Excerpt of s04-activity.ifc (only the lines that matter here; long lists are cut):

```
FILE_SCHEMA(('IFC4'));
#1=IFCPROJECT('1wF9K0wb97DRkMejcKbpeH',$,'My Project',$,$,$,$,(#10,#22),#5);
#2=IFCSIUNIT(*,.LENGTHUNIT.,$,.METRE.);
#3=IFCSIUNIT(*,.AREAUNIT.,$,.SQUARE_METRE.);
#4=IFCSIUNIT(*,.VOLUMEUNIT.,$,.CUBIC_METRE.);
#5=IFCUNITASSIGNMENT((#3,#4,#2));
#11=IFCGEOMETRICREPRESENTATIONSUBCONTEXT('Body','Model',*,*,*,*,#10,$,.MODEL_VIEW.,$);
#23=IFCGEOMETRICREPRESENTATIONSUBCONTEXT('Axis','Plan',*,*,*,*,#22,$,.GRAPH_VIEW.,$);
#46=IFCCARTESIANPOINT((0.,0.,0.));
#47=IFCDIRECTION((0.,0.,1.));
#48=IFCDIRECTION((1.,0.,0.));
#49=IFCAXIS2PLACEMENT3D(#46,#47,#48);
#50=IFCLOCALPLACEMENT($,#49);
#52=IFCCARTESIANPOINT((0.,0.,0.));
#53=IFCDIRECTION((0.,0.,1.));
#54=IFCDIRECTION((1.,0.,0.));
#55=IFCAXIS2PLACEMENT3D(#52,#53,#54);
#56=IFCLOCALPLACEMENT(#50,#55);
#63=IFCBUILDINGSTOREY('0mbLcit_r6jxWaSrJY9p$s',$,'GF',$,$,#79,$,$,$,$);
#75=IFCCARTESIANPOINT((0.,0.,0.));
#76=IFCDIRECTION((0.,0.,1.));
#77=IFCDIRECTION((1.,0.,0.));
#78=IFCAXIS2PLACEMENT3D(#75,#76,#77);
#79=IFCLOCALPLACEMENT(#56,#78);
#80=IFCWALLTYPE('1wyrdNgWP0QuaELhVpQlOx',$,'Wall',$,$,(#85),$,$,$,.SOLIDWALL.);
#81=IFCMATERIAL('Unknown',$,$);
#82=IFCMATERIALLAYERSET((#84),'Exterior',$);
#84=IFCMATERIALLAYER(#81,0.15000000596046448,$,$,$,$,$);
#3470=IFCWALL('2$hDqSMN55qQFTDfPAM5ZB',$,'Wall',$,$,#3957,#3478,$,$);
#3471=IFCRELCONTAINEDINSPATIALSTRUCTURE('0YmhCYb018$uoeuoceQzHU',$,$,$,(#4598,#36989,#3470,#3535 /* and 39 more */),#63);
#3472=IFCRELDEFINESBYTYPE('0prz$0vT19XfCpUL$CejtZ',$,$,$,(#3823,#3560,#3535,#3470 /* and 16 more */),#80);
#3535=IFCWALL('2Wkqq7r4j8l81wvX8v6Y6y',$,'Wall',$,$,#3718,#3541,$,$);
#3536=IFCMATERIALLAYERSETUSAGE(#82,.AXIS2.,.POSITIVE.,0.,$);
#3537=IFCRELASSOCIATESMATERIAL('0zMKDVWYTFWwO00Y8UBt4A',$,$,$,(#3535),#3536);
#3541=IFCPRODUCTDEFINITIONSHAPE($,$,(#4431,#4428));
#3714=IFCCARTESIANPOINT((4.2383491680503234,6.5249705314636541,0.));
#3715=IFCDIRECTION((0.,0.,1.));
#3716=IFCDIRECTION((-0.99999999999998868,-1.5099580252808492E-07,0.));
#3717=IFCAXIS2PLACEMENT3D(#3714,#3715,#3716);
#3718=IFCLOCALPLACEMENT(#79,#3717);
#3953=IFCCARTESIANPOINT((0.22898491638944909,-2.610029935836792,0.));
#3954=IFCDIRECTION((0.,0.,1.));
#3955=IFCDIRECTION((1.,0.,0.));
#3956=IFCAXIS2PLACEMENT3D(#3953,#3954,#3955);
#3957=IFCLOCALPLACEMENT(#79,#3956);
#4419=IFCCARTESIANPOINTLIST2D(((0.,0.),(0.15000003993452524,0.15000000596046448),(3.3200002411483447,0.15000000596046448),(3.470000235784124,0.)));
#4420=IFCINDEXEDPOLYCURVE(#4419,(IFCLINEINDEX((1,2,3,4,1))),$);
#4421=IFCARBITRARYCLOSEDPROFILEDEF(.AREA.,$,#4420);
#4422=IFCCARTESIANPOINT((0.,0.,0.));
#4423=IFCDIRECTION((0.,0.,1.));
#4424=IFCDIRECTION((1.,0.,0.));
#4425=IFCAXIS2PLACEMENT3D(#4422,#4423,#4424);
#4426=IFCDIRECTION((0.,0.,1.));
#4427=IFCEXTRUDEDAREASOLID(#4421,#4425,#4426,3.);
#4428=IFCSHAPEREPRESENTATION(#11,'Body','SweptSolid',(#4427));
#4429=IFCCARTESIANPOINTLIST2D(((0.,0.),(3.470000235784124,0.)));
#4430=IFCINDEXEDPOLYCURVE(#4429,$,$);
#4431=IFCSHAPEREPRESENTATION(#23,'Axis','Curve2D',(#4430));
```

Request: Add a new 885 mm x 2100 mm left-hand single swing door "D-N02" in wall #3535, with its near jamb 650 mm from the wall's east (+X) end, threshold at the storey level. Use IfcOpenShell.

```python
import numpy as np
import ifcopenshell
import ifcopenshell.api.feature
import ifcopenshell.api.geometry
import ifcopenshell.api.root
import ifcopenshell.api.spatial
import ifcopenshell.geom
import ifcopenshell.util.element
import ifcopenshell.util.placement
import ifcopenshell.util.representation
import ifcopenshell.util.shape
import ifcopenshell.util.unit

model = ifcopenshell.open("s04-activity.ifc")
unit_scale = ifcopenshell.util.unit.calculate_unit_scale(model)
settings = ifcopenshell.geom.settings()


def volume(element):
    """Net volume in cubic metres, openings subtracted."""
    shape = ifcopenshell.geom.create_shape(settings, element)
    return ifcopenshell.util.shape.get_volume(shape.geometry)


wall = model.by_guid("2Wkqq7r4j8l81wvX8v6Y6y")
storey = ifcopenshell.util.element.get_container(wall, ifc_class="IfcBuildingStorey")
context = ifcopenshell.util.representation.get_context(model, "Model", "Body", "MODEL_VIEW")
before = volume(wall)

width, height, from_end, sill = 0.885, 2.1, 0.65, 0.0  # metres

# The wall runs along its own X axis, and the end named is its -X end.
wall_shape = ifcopenshell.geom.create_shape(settings, wall)
x, y, z = ifcopenshell.util.shape.get_vertices(wall_shape.geometry).T
start = x.min() + from_end
face, thickness = float(y.min()), float(y.max() - y.min())
wall_matrix = ifcopenshell.util.placement.get_local_placement(wall.ObjectPlacement)
level = ifcopenshell.util.placement.get_local_placement(storey.ObjectPlacement)[2, 3]


def in_wall(x, y):
    """Placement at x, y metres in the wall's axes, at sill height."""
    matrix = wall_matrix.copy()
    matrix[:, 3] = wall_matrix @ np.array([x / unit_scale, y / unit_scale, 0.0, 1.0])
    matrix[2, 3] = level + sill / unit_scale
    return matrix


# Opening: a box that overshoots both wall faces by 50 mm.
opening = ifcopenshell.api.root.create_entity(model, ifc_class="IfcOpeningElement", predefined_type="OPENING")
box = ifcopenshell.api.geometry.add_wall_representation(
    model, context=context, length=width, height=height, thickness=thickness + 0.1
)
ifcopenshell.api.geometry.assign_representation(model, product=opening, representation=box)
ifcopenshell.api.geometry.edit_object_placement(model, product=opening, matrix=in_wall(start, face - 0.05), is_si=False)
ifcopenshell.api.feature.add_feature(model, feature=opening, element=wall)

door = ifcopenshell.api.root.create_entity(model, ifc_class="IfcDoor", name="D-N02", predefined_type="DOOR")
door.OverallWidth, door.OverallHeight = width / unit_scale, height / unit_scale
door.OperationType = "SINGLE_SWING_LEFT"
body = ifcopenshell.api.geometry.add_door_representation(
    model,
    context=context,
    overall_width=door.OverallWidth,
    overall_height=door.OverallHeight,
    operation_type="SINGLE_SWING_LEFT",
    lining_properties={"LiningDepth": thickness / unit_scale, "ThresholdDepth": thickness / unit_scale},
)
ifcopenshell.api.geometry.assign_representation(model, product=door, representation=body)
ifcopenshell.api.spatial.assign_container(model, products=[door], relating_structure=storey)
ifcopenshell.api.feature.add_filling(model, opening=opening, element=door)

# The lining spans the wall, so the door starts at the wall face.
ifcopenshell.api.geometry.edit_object_placement(model, product=door, matrix=in_wall(start, face), is_si=False)

after = volume(wall)

print(f"wall volume {before:.3f} -> {after:.3f} m3")

model.write("s04-activity_edited.ifc")
```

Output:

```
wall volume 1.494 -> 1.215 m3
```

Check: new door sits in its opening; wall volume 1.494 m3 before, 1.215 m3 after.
